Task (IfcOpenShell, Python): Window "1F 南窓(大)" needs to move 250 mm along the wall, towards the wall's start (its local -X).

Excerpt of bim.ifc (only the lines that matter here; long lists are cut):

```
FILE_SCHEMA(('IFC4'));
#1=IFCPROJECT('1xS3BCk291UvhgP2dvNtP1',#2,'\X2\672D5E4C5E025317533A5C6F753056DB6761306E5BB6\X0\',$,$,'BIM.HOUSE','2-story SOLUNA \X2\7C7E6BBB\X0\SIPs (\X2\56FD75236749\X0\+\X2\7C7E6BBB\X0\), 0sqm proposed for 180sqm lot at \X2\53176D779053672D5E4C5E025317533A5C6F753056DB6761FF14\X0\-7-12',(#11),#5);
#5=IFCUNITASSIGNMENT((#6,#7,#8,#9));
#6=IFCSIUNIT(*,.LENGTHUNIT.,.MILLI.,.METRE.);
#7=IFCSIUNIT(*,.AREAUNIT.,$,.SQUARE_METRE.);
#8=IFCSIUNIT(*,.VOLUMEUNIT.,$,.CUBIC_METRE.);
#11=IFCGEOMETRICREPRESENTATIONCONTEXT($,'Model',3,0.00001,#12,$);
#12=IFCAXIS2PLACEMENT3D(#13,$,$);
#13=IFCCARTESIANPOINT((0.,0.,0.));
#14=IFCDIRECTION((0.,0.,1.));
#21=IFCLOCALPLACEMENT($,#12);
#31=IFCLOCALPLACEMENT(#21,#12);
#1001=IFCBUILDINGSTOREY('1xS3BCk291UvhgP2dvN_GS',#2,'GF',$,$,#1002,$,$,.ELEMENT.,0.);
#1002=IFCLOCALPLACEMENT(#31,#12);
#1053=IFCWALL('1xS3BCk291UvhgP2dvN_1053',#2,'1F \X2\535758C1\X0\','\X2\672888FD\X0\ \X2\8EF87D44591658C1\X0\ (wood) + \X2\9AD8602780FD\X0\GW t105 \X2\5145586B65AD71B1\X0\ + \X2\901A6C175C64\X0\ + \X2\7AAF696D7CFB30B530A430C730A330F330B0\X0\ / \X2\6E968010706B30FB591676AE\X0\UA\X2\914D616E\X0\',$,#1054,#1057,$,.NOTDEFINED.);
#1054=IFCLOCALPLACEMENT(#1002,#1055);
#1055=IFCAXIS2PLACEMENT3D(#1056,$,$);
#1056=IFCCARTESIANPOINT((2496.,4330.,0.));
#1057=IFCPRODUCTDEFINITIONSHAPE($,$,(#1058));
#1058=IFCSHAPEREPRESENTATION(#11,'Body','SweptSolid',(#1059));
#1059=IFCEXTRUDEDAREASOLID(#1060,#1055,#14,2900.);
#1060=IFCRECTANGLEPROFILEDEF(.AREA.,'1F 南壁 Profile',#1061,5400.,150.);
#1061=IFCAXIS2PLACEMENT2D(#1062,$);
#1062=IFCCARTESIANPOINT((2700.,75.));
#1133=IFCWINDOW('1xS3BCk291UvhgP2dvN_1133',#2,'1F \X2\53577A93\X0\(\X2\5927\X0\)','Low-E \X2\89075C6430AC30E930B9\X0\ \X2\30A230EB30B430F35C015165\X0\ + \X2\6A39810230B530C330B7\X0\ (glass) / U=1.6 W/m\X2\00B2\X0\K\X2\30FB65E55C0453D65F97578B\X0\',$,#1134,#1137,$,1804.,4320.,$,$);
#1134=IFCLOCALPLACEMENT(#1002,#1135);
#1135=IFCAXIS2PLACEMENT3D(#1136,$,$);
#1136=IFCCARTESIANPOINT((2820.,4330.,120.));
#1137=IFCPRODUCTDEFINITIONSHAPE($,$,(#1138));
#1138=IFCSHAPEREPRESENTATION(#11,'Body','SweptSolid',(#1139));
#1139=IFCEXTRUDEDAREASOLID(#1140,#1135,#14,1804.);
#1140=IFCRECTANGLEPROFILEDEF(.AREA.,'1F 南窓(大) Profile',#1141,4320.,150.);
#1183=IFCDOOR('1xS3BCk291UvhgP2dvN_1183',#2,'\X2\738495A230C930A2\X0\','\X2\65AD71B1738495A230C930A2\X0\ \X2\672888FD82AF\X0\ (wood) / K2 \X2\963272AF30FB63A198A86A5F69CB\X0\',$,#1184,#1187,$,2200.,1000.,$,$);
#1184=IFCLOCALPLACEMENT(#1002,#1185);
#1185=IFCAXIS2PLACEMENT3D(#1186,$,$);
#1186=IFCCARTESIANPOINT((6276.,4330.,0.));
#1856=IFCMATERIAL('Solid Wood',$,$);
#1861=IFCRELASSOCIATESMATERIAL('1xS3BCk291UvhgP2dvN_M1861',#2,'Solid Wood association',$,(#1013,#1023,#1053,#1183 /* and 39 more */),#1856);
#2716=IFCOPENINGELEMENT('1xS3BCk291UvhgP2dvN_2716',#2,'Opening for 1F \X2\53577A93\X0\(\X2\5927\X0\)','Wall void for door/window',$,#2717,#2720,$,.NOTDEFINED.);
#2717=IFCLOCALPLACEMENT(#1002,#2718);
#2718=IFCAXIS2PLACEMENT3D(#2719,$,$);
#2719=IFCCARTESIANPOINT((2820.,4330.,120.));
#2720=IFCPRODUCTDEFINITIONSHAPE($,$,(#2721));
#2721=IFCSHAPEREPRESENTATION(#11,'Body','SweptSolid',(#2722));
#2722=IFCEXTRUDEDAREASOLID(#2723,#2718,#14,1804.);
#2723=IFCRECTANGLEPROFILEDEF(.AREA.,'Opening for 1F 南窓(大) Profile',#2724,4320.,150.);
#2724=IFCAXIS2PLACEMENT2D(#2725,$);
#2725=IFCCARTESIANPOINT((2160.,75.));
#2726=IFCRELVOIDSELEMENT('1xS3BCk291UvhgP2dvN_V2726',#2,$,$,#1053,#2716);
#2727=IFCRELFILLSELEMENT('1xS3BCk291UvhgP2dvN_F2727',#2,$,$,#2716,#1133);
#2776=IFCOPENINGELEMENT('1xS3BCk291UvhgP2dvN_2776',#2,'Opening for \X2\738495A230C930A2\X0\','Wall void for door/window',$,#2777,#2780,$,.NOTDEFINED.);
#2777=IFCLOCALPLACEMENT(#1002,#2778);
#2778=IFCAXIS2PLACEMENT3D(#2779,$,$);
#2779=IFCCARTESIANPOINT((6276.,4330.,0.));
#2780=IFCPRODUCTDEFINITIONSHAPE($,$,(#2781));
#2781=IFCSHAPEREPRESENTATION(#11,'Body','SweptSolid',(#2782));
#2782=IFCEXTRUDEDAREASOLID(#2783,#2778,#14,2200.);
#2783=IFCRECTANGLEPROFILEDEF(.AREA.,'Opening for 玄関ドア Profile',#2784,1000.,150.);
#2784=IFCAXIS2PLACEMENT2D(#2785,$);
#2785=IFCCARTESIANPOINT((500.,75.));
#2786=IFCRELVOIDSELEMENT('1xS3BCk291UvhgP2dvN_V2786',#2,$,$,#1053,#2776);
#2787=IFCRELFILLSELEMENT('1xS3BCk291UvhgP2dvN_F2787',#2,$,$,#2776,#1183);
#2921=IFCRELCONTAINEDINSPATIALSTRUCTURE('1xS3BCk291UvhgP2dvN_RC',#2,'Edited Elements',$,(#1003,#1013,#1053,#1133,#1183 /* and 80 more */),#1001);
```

```python
import ifcopenshell
import ifcopenshell.api.geometry
import ifcopenshell.util.placement

model = ifcopenshell.open("bim.ifc")

window = model.by_guid("1xS3BCk291UvhgP2dvN_1133")
opening = window.FillsVoids[0].RelatingOpeningElement
wall = opening.VoidsElements[0].RelatingBuildingElement

wall_matrix = ifcopenshell.util.placement.get_local_placement(wall.ObjectPlacement)
shift = wall_matrix[:3, 0] * -250.0
before = ifcopenshell.util.placement.get_local_placement(window.ObjectPlacement)[:3, 3].copy()

# The window is not placed relative to its opening, so move both.
for product in (opening, window):
    matrix = ifcopenshell.util.placement.get_local_placement(product.ObjectPlacement)
    matrix[:3, 3] += shift
    ifcopenshell.api.geometry.edit_object_placement(model, product=product, matrix=matrix, is_si=False)

after = ifcopenshell.util.placement.get_local_placement(window.ObjectPlacement)[:3, 3]
print("window moved by", (after - before).round(3) + 0.0)

model.write("bim_edited.ifc")
```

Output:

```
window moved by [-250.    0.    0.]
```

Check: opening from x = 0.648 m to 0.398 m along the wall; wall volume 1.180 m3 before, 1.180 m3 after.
